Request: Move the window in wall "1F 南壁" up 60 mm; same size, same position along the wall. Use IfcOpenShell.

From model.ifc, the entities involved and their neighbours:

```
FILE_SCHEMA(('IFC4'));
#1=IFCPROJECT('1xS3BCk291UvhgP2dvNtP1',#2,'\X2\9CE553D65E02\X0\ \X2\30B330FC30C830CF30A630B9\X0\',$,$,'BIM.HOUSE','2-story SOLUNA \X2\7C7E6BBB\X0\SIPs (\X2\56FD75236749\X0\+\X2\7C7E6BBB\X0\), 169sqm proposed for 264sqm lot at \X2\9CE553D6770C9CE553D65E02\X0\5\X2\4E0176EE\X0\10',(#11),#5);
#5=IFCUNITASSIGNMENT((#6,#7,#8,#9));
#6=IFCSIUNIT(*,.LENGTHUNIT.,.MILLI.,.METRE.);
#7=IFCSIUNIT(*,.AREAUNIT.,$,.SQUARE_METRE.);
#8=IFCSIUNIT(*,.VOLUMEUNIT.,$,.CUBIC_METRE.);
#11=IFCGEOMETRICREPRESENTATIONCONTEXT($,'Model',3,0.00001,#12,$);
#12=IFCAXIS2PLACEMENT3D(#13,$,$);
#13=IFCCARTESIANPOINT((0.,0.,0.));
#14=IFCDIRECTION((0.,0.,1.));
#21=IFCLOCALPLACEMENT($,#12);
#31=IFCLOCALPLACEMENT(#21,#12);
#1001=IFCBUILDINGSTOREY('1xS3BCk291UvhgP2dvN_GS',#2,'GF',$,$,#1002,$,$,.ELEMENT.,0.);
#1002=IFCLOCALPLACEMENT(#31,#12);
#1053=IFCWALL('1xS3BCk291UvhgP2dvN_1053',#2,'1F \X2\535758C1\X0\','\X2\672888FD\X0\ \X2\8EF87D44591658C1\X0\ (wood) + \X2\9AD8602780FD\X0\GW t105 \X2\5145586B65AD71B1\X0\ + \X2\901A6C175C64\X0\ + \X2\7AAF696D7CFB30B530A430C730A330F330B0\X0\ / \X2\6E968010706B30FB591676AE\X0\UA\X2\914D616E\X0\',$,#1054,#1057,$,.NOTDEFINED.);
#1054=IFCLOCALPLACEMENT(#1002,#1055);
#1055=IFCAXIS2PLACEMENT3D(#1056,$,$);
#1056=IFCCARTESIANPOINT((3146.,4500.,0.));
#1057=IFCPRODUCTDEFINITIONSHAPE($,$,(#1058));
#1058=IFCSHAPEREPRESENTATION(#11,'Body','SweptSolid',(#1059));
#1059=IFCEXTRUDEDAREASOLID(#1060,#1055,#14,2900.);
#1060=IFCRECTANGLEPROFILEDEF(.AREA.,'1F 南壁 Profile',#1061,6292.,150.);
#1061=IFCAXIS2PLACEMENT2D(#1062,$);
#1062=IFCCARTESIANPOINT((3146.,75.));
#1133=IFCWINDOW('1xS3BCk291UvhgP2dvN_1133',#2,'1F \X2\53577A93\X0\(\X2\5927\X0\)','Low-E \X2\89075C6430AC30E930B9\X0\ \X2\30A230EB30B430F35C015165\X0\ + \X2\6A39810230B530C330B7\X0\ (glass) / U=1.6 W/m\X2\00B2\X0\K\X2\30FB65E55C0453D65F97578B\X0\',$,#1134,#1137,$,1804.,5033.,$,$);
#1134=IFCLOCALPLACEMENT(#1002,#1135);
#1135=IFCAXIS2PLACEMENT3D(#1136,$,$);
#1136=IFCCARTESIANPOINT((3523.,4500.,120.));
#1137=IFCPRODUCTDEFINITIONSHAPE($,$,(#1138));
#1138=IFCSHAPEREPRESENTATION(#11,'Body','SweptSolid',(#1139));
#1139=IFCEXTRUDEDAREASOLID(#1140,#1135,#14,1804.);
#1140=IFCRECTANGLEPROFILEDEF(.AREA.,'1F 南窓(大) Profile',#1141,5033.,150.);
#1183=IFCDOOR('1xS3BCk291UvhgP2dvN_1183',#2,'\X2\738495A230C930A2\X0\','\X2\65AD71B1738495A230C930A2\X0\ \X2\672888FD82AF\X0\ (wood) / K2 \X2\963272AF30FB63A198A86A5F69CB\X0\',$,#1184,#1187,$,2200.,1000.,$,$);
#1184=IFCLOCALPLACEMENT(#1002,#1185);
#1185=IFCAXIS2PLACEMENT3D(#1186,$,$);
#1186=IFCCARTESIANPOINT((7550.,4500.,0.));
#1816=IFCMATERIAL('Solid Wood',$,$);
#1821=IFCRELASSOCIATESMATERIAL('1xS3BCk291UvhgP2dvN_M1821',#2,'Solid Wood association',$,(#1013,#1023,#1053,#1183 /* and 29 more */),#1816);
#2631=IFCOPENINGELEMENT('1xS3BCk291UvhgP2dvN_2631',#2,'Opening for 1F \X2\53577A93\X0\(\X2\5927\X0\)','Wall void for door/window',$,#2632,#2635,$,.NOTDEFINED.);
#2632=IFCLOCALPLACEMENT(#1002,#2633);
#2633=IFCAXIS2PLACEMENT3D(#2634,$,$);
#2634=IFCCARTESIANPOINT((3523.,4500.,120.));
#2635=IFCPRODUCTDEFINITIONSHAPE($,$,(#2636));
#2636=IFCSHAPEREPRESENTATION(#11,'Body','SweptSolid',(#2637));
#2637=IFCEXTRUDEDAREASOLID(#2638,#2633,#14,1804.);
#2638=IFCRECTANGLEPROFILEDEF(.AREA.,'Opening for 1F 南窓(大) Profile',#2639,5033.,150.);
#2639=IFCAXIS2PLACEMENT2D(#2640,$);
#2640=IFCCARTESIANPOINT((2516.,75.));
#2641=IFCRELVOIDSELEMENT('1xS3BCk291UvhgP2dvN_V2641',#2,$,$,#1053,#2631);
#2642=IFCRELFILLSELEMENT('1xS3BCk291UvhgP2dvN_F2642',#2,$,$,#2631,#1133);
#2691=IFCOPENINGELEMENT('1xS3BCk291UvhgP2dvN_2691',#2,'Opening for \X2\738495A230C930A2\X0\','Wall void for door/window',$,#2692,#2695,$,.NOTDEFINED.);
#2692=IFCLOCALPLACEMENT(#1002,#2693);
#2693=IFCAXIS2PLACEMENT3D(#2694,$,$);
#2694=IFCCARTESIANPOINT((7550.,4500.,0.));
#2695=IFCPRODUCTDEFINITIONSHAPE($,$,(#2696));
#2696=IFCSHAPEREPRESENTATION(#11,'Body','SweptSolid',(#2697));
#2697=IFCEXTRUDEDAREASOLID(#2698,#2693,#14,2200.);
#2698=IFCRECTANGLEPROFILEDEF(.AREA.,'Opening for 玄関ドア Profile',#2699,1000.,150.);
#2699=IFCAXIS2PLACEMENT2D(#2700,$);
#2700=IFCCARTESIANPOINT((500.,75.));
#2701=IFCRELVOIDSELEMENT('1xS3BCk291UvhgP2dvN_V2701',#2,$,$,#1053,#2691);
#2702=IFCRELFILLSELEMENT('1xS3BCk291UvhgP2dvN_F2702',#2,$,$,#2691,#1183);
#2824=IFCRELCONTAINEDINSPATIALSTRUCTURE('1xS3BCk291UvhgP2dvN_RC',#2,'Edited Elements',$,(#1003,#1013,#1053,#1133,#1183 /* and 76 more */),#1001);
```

```python
import numpy as np
import ifcopenshell
import ifcopenshell.api.geometry
import ifcopenshell.util.placement
import ifcopenshell.util.unit

model = ifcopenshell.open("model.ifc")
unit_scale = ifcopenshell.util.unit.calculate_unit_scale(model)

window = model.by_guid("1xS3BCk291UvhgP2dvN_1133")
opening = window.FillsVoids[0].RelatingOpeningElement
dz = 0.06 / unit_scale

shift = np.array([0.0, 0.0, dz])
# The window is not placed relative to its opening, so move both.
for product in (opening, window):
    matrix = ifcopenshell.util.placement.get_local_placement(product.ObjectPlacement)
    matrix[:3, 3] += shift
    ifcopenshell.api.geometry.edit_object_placement(model, product=product, matrix=matrix, is_si=False)

print(f"moved by {dz * unit_scale:+.3f} m")

model.write("model_updated.ifc")
```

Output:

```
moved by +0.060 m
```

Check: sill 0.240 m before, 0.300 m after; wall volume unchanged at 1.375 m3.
